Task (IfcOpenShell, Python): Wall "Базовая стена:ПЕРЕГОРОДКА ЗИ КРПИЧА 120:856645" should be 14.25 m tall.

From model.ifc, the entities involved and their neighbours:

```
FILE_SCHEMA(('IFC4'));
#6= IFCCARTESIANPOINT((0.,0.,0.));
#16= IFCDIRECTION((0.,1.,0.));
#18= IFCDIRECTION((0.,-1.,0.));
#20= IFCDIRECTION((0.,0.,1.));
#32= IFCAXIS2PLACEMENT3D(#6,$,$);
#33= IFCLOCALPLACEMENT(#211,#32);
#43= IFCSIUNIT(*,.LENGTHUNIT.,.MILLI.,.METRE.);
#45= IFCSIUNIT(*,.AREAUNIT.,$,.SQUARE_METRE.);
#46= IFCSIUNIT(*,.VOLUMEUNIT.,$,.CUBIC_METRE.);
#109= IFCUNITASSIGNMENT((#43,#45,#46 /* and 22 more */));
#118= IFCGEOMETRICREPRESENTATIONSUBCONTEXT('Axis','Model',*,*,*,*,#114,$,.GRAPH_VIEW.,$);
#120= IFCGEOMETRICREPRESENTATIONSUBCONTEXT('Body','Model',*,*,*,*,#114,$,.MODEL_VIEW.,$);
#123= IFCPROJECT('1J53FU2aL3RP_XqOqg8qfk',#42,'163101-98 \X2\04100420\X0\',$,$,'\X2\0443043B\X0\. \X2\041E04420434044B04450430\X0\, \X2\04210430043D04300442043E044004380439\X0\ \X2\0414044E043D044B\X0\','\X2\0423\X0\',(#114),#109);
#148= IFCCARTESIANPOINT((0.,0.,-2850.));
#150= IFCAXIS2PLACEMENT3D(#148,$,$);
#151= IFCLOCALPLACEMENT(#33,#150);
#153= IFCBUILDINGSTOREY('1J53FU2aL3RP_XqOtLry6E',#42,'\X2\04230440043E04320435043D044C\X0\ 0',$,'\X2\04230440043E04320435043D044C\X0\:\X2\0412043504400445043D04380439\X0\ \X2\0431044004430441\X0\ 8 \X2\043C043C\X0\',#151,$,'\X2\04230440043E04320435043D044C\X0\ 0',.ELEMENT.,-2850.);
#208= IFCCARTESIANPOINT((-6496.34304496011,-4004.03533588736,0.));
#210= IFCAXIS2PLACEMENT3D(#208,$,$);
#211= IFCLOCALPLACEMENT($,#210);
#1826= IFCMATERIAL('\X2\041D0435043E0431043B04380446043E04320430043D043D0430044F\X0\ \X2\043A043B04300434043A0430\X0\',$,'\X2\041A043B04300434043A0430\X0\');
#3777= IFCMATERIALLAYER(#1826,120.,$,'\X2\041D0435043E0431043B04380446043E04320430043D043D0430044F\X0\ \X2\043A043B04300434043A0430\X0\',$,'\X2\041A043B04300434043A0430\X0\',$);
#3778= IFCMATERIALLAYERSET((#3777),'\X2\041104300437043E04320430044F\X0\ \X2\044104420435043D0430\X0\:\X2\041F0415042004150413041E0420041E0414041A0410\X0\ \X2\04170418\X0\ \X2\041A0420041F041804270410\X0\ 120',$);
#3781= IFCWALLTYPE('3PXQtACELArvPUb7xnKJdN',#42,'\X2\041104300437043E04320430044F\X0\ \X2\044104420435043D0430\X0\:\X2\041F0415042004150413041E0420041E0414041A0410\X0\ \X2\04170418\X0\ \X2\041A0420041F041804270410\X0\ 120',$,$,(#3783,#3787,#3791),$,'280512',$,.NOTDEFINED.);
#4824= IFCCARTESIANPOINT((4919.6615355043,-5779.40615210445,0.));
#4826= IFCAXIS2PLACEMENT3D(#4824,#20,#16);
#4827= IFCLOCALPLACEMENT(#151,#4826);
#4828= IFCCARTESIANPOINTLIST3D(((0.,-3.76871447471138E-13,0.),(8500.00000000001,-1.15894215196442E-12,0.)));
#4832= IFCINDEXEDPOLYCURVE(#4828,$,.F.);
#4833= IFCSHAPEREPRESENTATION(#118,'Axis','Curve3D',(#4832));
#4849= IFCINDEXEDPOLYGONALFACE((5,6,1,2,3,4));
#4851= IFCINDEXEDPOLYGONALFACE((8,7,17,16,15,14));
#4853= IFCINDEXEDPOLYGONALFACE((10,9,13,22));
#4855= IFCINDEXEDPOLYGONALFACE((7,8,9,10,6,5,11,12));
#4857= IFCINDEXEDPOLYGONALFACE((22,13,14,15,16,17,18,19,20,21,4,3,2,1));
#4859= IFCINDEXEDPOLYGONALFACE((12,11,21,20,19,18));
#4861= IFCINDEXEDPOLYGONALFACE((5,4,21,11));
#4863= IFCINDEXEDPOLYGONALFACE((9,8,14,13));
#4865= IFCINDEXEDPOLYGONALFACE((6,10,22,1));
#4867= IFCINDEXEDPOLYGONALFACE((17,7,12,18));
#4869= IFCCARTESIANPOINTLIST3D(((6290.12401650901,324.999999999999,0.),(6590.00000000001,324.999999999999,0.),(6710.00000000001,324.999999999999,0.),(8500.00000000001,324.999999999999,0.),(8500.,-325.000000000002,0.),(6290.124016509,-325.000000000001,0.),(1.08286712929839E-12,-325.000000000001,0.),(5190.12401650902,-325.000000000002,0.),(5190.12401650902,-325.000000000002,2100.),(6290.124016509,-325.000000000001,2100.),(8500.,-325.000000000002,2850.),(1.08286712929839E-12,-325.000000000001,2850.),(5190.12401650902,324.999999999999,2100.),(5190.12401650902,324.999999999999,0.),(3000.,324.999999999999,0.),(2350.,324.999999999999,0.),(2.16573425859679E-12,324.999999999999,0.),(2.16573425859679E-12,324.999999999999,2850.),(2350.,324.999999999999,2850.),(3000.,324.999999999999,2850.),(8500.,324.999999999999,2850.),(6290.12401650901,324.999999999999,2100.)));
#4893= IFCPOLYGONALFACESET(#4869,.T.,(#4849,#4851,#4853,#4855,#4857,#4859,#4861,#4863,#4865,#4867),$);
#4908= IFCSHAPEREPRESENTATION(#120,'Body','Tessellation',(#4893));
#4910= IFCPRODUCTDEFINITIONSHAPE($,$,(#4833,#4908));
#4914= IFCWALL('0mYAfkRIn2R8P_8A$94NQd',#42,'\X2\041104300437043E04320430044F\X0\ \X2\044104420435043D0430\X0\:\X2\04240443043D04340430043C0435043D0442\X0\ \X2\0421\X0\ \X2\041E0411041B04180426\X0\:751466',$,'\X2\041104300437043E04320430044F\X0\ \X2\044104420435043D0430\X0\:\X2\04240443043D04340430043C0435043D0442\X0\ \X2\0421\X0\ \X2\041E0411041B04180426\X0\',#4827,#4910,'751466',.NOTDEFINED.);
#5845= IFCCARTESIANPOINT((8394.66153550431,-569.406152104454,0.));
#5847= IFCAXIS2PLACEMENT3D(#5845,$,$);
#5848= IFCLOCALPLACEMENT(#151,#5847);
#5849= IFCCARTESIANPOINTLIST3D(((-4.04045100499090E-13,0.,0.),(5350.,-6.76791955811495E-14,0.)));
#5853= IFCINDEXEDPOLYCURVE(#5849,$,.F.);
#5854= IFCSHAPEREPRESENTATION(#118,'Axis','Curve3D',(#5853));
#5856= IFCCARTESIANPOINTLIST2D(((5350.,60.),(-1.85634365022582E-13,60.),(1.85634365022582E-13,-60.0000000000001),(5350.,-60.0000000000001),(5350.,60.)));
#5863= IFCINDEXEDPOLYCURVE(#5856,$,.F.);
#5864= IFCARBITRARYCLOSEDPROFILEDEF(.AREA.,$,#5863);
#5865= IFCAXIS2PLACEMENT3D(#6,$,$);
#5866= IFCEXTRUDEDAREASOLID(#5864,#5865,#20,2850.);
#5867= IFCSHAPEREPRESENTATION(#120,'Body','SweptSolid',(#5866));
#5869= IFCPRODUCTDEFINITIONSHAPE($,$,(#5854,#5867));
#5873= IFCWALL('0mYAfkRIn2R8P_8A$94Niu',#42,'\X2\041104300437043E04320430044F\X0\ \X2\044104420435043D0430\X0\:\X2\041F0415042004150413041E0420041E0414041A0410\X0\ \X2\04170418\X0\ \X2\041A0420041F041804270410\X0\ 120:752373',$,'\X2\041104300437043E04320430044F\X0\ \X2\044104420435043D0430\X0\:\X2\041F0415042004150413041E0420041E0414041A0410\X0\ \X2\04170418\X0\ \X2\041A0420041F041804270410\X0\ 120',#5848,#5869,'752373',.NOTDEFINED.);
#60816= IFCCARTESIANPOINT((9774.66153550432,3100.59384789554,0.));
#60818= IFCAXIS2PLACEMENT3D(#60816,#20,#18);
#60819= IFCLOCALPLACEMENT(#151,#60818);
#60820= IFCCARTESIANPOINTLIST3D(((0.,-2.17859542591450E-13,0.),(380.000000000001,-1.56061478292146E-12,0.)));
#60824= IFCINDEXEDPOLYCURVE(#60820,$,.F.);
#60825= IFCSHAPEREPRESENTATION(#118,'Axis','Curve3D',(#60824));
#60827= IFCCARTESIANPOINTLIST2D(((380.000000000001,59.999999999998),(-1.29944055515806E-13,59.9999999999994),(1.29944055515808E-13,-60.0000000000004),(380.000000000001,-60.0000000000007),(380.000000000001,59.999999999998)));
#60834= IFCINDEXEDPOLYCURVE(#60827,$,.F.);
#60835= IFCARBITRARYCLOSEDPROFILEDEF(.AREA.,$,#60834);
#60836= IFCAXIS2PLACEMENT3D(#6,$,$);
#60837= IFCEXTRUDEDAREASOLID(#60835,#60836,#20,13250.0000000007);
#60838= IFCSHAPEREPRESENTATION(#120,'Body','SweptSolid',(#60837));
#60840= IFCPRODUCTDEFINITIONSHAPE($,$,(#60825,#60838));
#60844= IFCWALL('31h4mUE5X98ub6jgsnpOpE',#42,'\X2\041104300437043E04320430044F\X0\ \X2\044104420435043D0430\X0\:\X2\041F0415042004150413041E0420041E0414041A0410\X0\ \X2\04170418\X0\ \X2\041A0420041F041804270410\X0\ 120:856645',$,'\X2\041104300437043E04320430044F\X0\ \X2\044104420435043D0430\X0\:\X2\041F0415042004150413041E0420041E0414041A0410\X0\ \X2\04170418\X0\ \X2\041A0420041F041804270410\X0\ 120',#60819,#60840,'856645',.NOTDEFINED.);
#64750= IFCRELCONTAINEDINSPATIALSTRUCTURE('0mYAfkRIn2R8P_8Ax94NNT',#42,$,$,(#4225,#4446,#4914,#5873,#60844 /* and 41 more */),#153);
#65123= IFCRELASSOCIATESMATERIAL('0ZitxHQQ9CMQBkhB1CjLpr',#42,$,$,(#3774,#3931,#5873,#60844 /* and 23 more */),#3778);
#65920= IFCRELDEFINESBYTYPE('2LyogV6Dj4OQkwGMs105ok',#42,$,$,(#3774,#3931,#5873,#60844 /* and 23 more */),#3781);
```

```python
import ifcopenshell
import ifcopenshell.geom
import ifcopenshell.util.representation
import ifcopenshell.util.shape

model = ifcopenshell.open("model.ifc")
settings = ifcopenshell.geom.settings()


def volume(element):
    """Net volume in cubic metres, openings subtracted."""
    shape = ifcopenshell.geom.create_shape(settings, element)
    return ifcopenshell.util.shape.get_volume(shape.geometry)


wall = model.by_guid("31h4mUE5X98ub6jgsnpOpE")
before = volume(wall)

body = ifcopenshell.util.representation.get_representation(wall, "Model", "Body")
solid = body.Items[0]
old_height = solid.Depth
solid.Depth = 14250.0
after = volume(wall)

print(f"height {old_height:g} -> {solid.Depth:g}, volume {before:.3f} -> {after:.3f} m3")

model.write("model_updated.ifc")
```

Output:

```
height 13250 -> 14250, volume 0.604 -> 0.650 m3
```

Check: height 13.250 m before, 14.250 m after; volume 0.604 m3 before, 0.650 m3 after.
